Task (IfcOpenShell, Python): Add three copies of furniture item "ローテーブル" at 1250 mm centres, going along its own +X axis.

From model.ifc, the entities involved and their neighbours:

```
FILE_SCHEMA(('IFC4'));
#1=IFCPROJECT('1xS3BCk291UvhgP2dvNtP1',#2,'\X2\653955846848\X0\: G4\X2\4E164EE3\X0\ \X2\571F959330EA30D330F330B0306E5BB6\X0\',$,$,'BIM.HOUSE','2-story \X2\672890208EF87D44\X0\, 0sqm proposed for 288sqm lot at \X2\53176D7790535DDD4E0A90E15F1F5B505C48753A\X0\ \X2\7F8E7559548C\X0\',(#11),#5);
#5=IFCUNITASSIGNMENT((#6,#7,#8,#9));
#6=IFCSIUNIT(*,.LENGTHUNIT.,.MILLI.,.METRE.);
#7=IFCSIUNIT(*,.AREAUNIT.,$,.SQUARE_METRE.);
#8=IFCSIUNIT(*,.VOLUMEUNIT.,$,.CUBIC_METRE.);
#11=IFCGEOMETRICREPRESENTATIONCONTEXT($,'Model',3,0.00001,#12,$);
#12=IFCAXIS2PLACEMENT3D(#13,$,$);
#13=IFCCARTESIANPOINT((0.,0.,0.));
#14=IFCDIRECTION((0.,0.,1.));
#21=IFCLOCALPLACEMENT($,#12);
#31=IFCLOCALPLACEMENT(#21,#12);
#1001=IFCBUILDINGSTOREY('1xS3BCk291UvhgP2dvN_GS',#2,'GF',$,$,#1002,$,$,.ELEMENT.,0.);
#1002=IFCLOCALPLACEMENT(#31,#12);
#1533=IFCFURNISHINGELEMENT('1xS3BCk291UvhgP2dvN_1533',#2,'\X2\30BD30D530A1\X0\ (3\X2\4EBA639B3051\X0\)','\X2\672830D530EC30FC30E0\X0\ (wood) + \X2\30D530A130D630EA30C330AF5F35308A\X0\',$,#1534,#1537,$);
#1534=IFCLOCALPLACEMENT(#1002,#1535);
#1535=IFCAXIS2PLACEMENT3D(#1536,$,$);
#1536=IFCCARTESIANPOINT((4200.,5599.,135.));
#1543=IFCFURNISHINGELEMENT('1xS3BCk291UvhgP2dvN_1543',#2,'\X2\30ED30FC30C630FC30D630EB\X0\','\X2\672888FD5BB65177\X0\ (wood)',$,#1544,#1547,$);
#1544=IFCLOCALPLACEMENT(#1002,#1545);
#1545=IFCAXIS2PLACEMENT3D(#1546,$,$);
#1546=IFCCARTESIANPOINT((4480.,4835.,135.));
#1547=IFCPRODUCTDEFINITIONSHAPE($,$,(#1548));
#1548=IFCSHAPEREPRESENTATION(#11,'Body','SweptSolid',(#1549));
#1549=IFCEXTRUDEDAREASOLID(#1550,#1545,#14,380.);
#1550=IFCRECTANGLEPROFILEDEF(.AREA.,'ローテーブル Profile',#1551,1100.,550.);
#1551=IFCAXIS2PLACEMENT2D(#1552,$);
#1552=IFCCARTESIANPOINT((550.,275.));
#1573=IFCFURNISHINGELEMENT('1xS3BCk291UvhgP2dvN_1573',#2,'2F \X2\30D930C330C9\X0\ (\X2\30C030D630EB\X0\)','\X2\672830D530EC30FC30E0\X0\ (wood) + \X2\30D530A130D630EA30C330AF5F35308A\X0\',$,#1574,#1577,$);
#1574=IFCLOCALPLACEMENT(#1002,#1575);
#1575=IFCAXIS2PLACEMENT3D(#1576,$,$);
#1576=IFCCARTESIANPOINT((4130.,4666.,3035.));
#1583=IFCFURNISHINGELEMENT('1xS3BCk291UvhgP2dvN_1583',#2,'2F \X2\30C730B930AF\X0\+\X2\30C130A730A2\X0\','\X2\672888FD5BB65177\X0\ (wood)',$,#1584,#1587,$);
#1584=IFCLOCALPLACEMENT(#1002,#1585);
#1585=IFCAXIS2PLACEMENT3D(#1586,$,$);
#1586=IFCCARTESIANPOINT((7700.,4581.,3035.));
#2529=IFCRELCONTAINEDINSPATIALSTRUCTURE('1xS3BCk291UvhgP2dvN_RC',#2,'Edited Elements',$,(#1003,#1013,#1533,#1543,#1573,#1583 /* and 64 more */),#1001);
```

```python
import ifcopenshell
import ifcopenshell.api.geometry
import ifcopenshell.api.root
import ifcopenshell.util.element
import ifcopenshell.util.placement
import ifcopenshell.util.unit

model = ifcopenshell.open("model.ifc")
unit_scale = ifcopenshell.util.unit.calculate_unit_scale(model)


def reuse_history(source, copy):
    """copy_class also copies each property set's owner history, people and application; keep the originals."""
    for rel in copy.IsDefinedBy:
        if rel.is_a("IfcRelDefinesByProperties") and (history := rel.RelatingPropertyDefinition.OwnerHistory):
            rel.RelatingPropertyDefinition.OwnerHistory = source.OwnerHistory
            ifcopenshell.util.element.remove_deep2(model, history)


source = model.by_guid("1xS3BCk291UvhgP2dvN_1543")
base = ifcopenshell.util.placement.get_local_placement(source.ObjectPlacement)
step = base[:3, 0] * 1.25 / unit_scale

for i in range(1, 4):
    copy = ifcopenshell.api.root.copy_class(model, product=source)
    copy.Representation = ifcopenshell.util.element.copy_deep(
        model, source.Representation, exclude=["IfcGeometricRepresentationContext", "IfcRepresentationMap"]
    )
    reuse_history(source, copy)
    matrix = base.copy()
    matrix[:3, 3] += i * step
    print("added at", matrix[:3, 3].round(3) + 0.0)
    ifcopenshell.api.geometry.edit_object_placement(model, product=copy, matrix=matrix, is_si=False)

model.write("model_v2.ifc")
```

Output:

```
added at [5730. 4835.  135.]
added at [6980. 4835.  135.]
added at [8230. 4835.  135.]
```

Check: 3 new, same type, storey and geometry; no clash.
